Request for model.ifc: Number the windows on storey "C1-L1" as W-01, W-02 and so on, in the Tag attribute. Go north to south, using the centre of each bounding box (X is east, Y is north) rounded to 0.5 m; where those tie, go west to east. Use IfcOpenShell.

First a look at what the model holds.

```python
import ifcopenshell
import ifcopenshell.util.element
import ifcopenshell.util.placement

model = ifcopenshell.open("model.ifc")
print(model.schema)
storey = next(s for s in model.by_type("IfcBuildingStorey") if s.Name == "C1-L1")
windows = [e for e in ifcopenshell.util.element.get_decomposition(storey) if e.is_a("IfcWindow")]
for e in sorted(windows, key=lambda e: e.id()):
    origin = ifcopenshell.util.placement.get_local_placement(e.ObjectPlacement)[:3, 3]
    print(e.id(), e.Tag, e.Name, origin.round(2) + 0.0, sep=" | ")
```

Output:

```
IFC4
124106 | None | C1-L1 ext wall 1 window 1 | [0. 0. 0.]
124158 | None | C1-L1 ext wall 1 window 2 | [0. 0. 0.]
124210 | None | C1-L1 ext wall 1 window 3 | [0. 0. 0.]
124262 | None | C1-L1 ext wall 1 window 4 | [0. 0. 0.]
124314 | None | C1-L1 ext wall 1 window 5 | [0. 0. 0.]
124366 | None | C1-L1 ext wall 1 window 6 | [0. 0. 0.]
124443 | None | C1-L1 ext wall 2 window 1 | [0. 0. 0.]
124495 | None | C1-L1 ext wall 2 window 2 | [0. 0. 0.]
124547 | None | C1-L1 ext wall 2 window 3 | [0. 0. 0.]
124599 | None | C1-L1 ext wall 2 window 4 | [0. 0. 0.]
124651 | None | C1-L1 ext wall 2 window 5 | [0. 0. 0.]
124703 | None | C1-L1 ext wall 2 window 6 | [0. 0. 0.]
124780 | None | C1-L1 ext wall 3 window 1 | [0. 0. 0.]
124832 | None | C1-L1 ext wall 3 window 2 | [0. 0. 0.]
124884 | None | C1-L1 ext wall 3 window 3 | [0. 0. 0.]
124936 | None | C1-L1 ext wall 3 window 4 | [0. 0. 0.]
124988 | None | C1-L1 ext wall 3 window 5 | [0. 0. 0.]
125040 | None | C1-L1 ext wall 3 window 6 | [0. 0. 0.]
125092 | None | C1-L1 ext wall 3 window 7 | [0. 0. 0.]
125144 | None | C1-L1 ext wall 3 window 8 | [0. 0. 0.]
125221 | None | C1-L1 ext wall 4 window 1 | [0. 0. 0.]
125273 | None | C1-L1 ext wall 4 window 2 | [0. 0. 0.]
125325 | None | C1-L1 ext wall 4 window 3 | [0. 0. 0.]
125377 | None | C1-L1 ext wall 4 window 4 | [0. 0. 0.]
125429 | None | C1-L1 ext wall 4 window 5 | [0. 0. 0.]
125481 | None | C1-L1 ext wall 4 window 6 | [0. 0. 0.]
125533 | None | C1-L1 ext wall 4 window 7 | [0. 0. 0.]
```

```python
import ifcopenshell
import ifcopenshell.geom
import ifcopenshell.util.element
import ifcopenshell.util.shape

model = ifcopenshell.open("model.ifc")
settings = ifcopenshell.geom.settings()
settings.set("use-world-coords", True)


def centre(element):
    shape = ifcopenshell.geom.create_shape(settings, element)
    return ifcopenshell.util.shape.get_bbox_centroid(shape.geometry)


storey = next(s for s in model.by_type("IfcBuildingStorey") if s.Name == "C1-L1")
windows = [e for e in ifcopenshell.util.element.get_decomposition(storey) if e.is_a("IfcWindow")]

# Insertion points can sit at a corner or the storey origin, so sort by the geometry (in metres).
centres = {e: centre(e) for e in windows}
windows.sort(key=lambda e: (-round(centres[e][1] / 0.5), centres[e][0]))

for i, e in enumerate(windows, start=1):
    number = f"W-{i:02d}"
    e.Tag = number
    print(e.id(), number)

model.write("model-out.ifc")
```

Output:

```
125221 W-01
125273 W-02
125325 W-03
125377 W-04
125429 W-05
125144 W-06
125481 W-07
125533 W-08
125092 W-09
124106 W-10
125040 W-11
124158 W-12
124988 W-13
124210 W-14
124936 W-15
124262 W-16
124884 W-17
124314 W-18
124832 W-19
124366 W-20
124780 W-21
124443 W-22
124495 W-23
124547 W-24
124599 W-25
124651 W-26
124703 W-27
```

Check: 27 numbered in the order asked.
